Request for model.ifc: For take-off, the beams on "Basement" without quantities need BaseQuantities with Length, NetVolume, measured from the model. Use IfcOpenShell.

First a look at what the model holds.

```python
import ifcopenshell
import ifcopenshell.util.element
import ifcopenshell.util.unit

model = ifcopenshell.open("model.ifc")
print(model.schema)
for unit_type in ("LENGTHUNIT", "AREAUNIT", "VOLUMEUNIT"):
    print(unit_type, ifcopenshell.util.unit.calculate_unit_scale(model, unit_type))
storey = next(s for s in model.by_type("IfcBuildingStorey") if s.Name == "Basement")
beams = [e for e in ifcopenshell.util.element.get_decomposition(storey) if e.is_a("IfcBeam")]
for e in sorted(beams, key=lambda e: e.id()):
    print(e.id(), e.is_a(), e.Name, list(ifcopenshell.util.element.get_psets(e, qtos_only=True)), sep=" | ")
```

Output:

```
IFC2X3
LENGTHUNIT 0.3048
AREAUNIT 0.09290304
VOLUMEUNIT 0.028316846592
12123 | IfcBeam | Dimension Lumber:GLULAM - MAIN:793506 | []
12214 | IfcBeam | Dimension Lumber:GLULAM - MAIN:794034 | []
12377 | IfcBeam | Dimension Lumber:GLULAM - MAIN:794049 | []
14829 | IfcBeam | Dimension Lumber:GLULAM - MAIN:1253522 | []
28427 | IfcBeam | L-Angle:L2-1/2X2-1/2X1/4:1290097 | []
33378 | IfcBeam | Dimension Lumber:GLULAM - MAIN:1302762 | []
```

```python
import ifcopenshell
import ifcopenshell.api.pset
import ifcopenshell.geom
import ifcopenshell.util.element
import ifcopenshell.util.shape
import ifcopenshell.util.unit

model = ifcopenshell.open("model.ifc")
unit_scale = ifcopenshell.util.unit.calculate_unit_scale(model)
volume_scale = ifcopenshell.util.unit.calculate_unit_scale(model, "VOLUMEUNIT")
settings = ifcopenshell.geom.settings()

storey = next(s for s in model.by_type("IfcBuildingStorey") if s.Name == "Basement")
beams = [e for e in ifcopenshell.util.element.get_decomposition(storey) if e.is_a("IfcBeam")]

for e in sorted(beams, key=lambda e: e.id()):
    if ifcopenshell.util.element.get_psets(e, qtos_only=True, should_inherit=False):
        continue
    # Geometry comes back in metres, in the element's own axes.
    shape = ifcopenshell.geom.create_shape(settings, e)
    values = {
        "Length": ifcopenshell.util.shape.get_max_xyz(shape.geometry) / unit_scale,
        "NetVolume": ifcopenshell.util.shape.get_volume(shape.geometry) / volume_scale,
    }
    qto = ifcopenshell.api.pset.add_qto(model, product=e, name="BaseQuantities")
    ifcopenshell.api.pset.edit_qto(model, qto=qto, properties=values)
    print(e.id(), {k: round(v, 3) for k, v in values.items()})

model.write("model_rev.ifc")
```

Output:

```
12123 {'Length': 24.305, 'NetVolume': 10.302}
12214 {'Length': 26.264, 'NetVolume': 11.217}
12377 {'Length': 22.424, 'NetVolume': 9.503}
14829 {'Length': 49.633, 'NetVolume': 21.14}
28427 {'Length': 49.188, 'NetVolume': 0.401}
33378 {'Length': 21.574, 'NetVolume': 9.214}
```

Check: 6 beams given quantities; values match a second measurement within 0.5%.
